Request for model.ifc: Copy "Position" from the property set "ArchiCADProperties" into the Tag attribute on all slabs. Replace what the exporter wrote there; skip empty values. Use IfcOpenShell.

First a look at what the model holds.

```python
import ifcopenshell
import ifcopenshell.util.element

model = ifcopenshell.open("model.ifc")
print(model.schema)
slabs = model.by_type("IfcSlab")
print(len(slabs), "slabs")
for e in slabs[:8]:
    source = ifcopenshell.util.element.get_pset(e, "ArchiCADProperties", "Position")
    target = e.Tag
    print(e.id(), repr(source), repr(target), sep=" | ")
```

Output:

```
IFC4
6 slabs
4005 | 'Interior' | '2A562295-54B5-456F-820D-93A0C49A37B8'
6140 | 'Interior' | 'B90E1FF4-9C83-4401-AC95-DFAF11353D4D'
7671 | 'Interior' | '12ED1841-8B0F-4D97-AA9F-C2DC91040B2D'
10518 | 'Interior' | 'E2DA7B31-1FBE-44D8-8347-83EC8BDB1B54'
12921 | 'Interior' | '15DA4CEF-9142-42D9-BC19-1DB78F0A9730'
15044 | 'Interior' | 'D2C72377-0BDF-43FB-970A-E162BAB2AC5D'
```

```python
import ifcopenshell
import ifcopenshell.util.element

model = ifcopenshell.open("model.ifc")

count = 0
for e in model.by_type("IfcSlab"):
    value = ifcopenshell.util.element.get_pset(e, "ArchiCADProperties", "Position")
    current = e.Tag
    if not value or not value.strip() or current == value:
        continue
    e.Tag = value
    count += 1

print(count, "slabs updated")

model.write("model_updated.ifc")
```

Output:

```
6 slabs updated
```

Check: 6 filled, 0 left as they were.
